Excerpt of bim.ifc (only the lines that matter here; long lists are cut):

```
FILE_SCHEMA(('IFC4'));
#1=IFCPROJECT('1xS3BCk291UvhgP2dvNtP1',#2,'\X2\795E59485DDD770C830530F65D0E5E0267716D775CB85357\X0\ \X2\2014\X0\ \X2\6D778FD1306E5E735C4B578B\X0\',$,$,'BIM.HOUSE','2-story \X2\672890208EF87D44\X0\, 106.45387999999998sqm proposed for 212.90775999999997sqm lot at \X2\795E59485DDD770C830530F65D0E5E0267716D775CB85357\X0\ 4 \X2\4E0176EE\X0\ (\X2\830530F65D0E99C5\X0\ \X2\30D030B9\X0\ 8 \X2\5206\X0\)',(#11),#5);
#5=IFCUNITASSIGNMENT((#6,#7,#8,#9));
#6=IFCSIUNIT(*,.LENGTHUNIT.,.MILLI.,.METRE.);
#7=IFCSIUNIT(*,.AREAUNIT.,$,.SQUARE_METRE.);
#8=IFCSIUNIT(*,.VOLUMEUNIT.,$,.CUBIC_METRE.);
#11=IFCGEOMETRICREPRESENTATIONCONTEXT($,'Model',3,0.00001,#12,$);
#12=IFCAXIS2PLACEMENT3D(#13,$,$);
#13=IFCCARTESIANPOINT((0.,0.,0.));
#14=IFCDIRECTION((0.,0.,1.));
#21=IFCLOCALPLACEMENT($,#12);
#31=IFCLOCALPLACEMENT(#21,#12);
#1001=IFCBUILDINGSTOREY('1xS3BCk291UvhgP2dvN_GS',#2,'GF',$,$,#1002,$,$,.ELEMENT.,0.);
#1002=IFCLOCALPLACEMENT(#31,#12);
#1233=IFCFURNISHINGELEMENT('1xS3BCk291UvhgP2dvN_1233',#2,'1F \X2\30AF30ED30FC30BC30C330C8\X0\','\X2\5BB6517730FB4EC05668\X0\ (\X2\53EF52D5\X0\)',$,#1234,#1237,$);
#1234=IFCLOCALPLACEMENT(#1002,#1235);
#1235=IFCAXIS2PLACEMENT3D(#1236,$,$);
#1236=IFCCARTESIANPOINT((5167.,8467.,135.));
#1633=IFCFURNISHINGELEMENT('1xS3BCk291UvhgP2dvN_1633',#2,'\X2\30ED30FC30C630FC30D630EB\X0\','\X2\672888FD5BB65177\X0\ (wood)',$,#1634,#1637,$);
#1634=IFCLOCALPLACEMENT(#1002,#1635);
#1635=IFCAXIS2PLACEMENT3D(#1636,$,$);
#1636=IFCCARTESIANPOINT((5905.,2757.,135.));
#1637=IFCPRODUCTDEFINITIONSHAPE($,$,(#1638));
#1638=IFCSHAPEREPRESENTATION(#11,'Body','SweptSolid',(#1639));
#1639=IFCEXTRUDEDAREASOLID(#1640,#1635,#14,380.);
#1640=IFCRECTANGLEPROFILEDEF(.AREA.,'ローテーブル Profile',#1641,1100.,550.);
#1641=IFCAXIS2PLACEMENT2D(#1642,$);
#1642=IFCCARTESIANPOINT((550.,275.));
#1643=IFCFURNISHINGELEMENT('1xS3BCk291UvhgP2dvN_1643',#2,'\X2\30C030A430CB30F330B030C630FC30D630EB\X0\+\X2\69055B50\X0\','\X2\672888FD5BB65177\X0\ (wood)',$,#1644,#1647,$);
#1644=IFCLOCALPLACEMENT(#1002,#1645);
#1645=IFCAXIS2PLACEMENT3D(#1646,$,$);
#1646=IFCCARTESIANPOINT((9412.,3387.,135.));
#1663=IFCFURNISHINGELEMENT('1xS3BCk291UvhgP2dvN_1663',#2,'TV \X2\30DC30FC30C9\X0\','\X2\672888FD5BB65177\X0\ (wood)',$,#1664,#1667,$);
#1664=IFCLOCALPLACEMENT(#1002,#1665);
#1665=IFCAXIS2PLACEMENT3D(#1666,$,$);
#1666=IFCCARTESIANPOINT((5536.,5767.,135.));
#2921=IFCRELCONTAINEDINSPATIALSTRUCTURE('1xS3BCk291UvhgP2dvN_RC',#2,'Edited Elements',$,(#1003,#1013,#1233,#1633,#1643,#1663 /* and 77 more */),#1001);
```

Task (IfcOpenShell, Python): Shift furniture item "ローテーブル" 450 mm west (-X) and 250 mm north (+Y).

```python
import ifcopenshell
import ifcopenshell.api.geometry
import ifcopenshell.util.placement

model = ifcopenshell.open("bim.ifc")

item = model.by_id(1633)
matrix = ifcopenshell.util.placement.get_local_placement(item.ObjectPlacement)
matrix[0, 3] -= 450.0
matrix[1, 3] += 250.0
ifcopenshell.api.geometry.edit_object_placement(model, product=item, matrix=matrix, is_si=False)

print(ifcopenshell.util.placement.get_local_placement(item.ObjectPlacement).round(3) + 0.0)

model.write("bim-out.ifc")
```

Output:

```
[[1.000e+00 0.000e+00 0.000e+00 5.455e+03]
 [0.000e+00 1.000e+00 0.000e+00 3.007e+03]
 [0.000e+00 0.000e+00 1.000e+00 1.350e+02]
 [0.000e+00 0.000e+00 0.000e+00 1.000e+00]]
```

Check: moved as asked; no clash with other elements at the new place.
